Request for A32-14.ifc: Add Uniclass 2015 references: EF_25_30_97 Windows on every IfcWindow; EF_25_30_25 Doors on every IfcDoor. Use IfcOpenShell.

First a look at what the model holds.

```python
import ifcopenshell

model = ifcopenshell.open("A32-14.ifc")
print(model.schema)
print("classifications:", [c.Name for c in model.by_type("IfcClassification")])
for ifc_class in ("IfcDoor", "IfcRoof", "IfcStair", "IfcWall", "IfcWindow"):
    print(ifc_class, len(model.by_type(ifc_class)))
```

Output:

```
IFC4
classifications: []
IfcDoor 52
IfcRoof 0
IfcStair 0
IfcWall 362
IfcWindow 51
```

```python
import ifcopenshell
import ifcopenshell.api.classification

model = ifcopenshell.open("A32-14.ifc")

system = ifcopenshell.api.classification.add_classification(model, classification="Uniclass 2015")

codes = {
    "IfcWindow": ("EF_25_30_97", "Windows"),
    "IfcDoor": ("EF_25_30_25", "Doors"),
}
for ifc_class, (code, name) in codes.items():
    products = model.by_type(ifc_class)
    ifcopenshell.api.classification.add_reference(
        model, products=products, classification=system, identification=code, name=name
    )
    print(code, len(products))

model.write("A32-14_edited.ifc")
```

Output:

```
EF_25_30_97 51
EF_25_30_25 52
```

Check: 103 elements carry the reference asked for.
